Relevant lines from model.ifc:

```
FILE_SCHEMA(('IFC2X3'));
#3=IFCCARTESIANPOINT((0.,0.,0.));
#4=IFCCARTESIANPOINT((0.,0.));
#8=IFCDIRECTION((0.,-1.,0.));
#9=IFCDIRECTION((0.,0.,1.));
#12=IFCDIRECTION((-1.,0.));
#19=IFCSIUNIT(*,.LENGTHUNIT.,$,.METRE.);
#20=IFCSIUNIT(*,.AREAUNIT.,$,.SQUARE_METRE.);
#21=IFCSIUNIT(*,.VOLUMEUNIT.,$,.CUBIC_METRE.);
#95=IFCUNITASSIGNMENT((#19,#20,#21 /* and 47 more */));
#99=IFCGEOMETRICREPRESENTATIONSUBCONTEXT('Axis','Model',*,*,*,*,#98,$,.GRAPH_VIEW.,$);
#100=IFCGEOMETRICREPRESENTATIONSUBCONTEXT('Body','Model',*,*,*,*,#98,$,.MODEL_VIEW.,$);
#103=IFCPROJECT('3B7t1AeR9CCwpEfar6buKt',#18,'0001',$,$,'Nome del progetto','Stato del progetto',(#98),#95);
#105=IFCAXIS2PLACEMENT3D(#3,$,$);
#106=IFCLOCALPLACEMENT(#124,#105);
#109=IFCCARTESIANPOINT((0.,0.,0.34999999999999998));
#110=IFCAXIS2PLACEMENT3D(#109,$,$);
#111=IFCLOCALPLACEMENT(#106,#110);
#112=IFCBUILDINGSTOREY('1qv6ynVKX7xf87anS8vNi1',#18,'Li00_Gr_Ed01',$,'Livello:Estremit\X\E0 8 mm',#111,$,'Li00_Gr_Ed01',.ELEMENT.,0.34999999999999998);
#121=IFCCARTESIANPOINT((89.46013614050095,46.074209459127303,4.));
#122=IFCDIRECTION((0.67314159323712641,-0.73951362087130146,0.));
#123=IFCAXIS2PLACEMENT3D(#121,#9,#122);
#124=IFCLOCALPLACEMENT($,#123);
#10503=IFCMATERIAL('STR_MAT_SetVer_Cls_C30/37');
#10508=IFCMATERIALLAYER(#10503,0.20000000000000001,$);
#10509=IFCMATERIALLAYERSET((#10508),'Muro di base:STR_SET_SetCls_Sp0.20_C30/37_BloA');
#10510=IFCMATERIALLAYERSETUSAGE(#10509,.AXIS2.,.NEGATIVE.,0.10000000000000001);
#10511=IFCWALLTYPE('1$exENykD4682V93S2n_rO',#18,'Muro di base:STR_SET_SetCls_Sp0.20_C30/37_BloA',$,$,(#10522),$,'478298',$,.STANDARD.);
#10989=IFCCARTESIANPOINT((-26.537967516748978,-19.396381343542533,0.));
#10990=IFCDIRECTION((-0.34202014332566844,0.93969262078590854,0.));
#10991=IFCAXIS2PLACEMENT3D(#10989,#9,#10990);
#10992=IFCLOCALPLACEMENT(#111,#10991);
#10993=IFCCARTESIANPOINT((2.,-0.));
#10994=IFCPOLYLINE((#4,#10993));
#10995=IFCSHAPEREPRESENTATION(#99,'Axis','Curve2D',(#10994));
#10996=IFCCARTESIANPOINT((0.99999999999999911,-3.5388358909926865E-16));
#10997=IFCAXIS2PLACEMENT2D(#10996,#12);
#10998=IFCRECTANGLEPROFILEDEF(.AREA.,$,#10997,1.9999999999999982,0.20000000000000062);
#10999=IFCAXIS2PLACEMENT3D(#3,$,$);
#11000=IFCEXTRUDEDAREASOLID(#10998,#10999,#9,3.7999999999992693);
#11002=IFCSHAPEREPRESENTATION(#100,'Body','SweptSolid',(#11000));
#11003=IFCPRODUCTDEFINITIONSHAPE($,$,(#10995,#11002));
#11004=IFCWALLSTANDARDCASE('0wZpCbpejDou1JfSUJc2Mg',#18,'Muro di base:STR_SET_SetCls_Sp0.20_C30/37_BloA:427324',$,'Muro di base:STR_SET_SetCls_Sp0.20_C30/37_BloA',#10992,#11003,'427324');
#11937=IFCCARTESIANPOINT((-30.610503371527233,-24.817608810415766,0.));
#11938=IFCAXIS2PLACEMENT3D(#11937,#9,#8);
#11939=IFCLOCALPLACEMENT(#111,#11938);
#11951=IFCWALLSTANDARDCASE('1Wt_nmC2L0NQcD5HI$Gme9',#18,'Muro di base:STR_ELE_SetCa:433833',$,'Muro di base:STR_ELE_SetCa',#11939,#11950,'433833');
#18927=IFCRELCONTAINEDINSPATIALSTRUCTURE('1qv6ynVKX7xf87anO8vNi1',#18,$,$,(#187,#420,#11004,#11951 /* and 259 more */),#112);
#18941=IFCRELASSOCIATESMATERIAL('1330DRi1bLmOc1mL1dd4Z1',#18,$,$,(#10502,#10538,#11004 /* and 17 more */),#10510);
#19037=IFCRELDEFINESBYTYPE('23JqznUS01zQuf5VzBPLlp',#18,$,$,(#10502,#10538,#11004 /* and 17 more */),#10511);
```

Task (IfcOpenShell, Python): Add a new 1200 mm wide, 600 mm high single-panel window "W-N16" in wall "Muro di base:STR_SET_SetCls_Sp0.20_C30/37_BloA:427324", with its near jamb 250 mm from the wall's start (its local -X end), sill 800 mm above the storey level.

```python
import numpy as np
import ifcopenshell
import ifcopenshell.api.feature
import ifcopenshell.api.geometry
import ifcopenshell.api.root
import ifcopenshell.api.spatial
import ifcopenshell.api.type
import ifcopenshell.geom
import ifcopenshell.util.element
import ifcopenshell.util.placement
import ifcopenshell.util.representation
import ifcopenshell.util.shape
import ifcopenshell.util.unit

model = ifcopenshell.open("model.ifc")
unit_scale = ifcopenshell.util.unit.calculate_unit_scale(model)
settings = ifcopenshell.geom.settings()


def volume(element):
    """Net volume in cubic metres, openings subtracted."""
    shape = ifcopenshell.geom.create_shape(settings, element)
    return ifcopenshell.util.shape.get_volume(shape.geometry)


wall = model.by_id(11004)
storey = ifcopenshell.util.element.get_container(wall, ifc_class="IfcBuildingStorey")
context = ifcopenshell.util.representation.get_context(model, "Model", "Body", "MODEL_VIEW")
before = volume(wall)

width, height, from_end, sill = 1.2, 0.6, 0.25, 0.8  # metres

# The wall runs along its own X axis, and the end named is its -X end.
wall_shape = ifcopenshell.geom.create_shape(settings, wall)
x, y, z = ifcopenshell.util.shape.get_vertices(wall_shape.geometry).T
start = x.min() + from_end
face, thickness = float(y.min()), float(y.max() - y.min())
wall_matrix = ifcopenshell.util.placement.get_local_placement(wall.ObjectPlacement)
level = ifcopenshell.util.placement.get_local_placement(storey.ObjectPlacement)[2, 3]


def in_wall(x, y):
    """Placement at x, y metres in the wall's axes, at sill height."""
    matrix = wall_matrix.copy()
    matrix[:, 3] = wall_matrix @ np.array([x / unit_scale, y / unit_scale, 0.0, 1.0])
    matrix[2, 3] = level + sill / unit_scale
    return matrix


# Opening: a box that overshoots both wall faces by 50 mm.
opening = ifcopenshell.api.root.create_entity(model, ifc_class="IfcOpeningElement")
box = ifcopenshell.api.geometry.add_wall_representation(
    model, context=context, length=width, height=height, thickness=thickness + 0.1
)
ifcopenshell.api.geometry.assign_representation(model, product=opening, representation=box)
ifcopenshell.api.geometry.edit_object_placement(model, product=opening, matrix=in_wall(start, face - 0.05), is_si=False)
ifcopenshell.api.feature.add_feature(model, feature=opening, element=wall)

window = ifcopenshell.api.root.create_entity(model, ifc_class="IfcWindow", name="W-N16")
window.OverallWidth, window.OverallHeight = width / unit_scale, height / unit_scale
body = ifcopenshell.api.geometry.add_window_representation(
    model,
    context=context,
    overall_width=window.OverallWidth,
    overall_height=window.OverallHeight,
    partition_type="SINGLE_PANEL",
)
ifcopenshell.api.geometry.assign_representation(model, product=window, representation=body)
ifcopenshell.api.spatial.assign_container(model, products=[window], relating_structure=storey)
fills = ifcopenshell.api.feature.add_filling(model, opening=opening, element=window)
fills.OwnerHistory = window.OwnerHistory  # required in IFC2X3

# IFC2X3 keeps the operation on the window style.
style = ifcopenshell.api.root.create_entity(model, ifc_class="IfcWindowStyle", name="W-N16")
style.OperationType, style.ConstructionType = "SINGLE_PANEL", "NOTDEFINED"
style.ParameterTakesPrecedence = style.Sizeable = False
ifcopenshell.api.type.assign_type(model, related_objects=[window], relating_type=style)

# Centre the window in the wall's thickness.
ifcopenshell.api.geometry.edit_object_placement(model, product=window, matrix=in_wall(start, face), is_si=False)
window_shape = ifcopenshell.geom.create_shape(settings, window)
depth = ifcopenshell.util.shape.get_vertices(window_shape.geometry)[:, 1]
offset = face + thickness / 2 - (depth.min() + depth.max()) / 2
ifcopenshell.api.geometry.edit_object_placement(model, product=window, matrix=in_wall(start, offset), is_si=False)

after = volume(wall)

print(f"wall volume {before:.3f} -> {after:.3f} m3")

model.write("model_edited.ifc")
```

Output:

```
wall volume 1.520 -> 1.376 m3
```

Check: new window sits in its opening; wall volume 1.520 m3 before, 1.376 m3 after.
